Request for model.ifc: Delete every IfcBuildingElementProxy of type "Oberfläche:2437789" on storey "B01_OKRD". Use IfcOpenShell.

First a look at what the model holds.

```python
import ifcopenshell
import ifcopenshell.util.element

model = ifcopenshell.open("model.ifc")
print(model.schema)
storey = next(s for s in model.by_type("IfcBuildingStorey") if s.Name == "B01_OKRD")
proxies = [e for e in ifcopenshell.util.element.get_decomposition(storey) if e.is_a("IfcBuildingElementProxy")]
seen = {}
for e in proxies:
    element_type = ifcopenshell.util.element.get_type(e)
    name = element_type.Name if element_type not in (None, e) else None
    seen[name] = seen.get(name, 0) + 1
for name, count in sorted(seen.items(), key=str):
    print(count, "x", name)
```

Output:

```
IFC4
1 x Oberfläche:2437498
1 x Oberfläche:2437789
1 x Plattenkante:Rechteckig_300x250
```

```python
import ifcopenshell
import ifcopenshell.api.root
import ifcopenshell.util.element

model = ifcopenshell.open("model.ifc")

storey = next(s for s in model.by_type("IfcBuildingStorey") if s.Name == "B01_OKRD")
proxies = [e for e in ifcopenshell.util.element.get_decomposition(storey) if e.is_a("IfcBuildingElementProxy")]
targets = [e for e in proxies if (t := ifcopenshell.util.element.get_type(e)) not in (None, e) and t.Name == "Oberfläche:2437789"]

for e in targets:
    ifcopenshell.api.root.remove_product(model, product=e)
print(len(targets), "removed")

model.write("model_rev.ifc")
```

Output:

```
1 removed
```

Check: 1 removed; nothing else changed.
